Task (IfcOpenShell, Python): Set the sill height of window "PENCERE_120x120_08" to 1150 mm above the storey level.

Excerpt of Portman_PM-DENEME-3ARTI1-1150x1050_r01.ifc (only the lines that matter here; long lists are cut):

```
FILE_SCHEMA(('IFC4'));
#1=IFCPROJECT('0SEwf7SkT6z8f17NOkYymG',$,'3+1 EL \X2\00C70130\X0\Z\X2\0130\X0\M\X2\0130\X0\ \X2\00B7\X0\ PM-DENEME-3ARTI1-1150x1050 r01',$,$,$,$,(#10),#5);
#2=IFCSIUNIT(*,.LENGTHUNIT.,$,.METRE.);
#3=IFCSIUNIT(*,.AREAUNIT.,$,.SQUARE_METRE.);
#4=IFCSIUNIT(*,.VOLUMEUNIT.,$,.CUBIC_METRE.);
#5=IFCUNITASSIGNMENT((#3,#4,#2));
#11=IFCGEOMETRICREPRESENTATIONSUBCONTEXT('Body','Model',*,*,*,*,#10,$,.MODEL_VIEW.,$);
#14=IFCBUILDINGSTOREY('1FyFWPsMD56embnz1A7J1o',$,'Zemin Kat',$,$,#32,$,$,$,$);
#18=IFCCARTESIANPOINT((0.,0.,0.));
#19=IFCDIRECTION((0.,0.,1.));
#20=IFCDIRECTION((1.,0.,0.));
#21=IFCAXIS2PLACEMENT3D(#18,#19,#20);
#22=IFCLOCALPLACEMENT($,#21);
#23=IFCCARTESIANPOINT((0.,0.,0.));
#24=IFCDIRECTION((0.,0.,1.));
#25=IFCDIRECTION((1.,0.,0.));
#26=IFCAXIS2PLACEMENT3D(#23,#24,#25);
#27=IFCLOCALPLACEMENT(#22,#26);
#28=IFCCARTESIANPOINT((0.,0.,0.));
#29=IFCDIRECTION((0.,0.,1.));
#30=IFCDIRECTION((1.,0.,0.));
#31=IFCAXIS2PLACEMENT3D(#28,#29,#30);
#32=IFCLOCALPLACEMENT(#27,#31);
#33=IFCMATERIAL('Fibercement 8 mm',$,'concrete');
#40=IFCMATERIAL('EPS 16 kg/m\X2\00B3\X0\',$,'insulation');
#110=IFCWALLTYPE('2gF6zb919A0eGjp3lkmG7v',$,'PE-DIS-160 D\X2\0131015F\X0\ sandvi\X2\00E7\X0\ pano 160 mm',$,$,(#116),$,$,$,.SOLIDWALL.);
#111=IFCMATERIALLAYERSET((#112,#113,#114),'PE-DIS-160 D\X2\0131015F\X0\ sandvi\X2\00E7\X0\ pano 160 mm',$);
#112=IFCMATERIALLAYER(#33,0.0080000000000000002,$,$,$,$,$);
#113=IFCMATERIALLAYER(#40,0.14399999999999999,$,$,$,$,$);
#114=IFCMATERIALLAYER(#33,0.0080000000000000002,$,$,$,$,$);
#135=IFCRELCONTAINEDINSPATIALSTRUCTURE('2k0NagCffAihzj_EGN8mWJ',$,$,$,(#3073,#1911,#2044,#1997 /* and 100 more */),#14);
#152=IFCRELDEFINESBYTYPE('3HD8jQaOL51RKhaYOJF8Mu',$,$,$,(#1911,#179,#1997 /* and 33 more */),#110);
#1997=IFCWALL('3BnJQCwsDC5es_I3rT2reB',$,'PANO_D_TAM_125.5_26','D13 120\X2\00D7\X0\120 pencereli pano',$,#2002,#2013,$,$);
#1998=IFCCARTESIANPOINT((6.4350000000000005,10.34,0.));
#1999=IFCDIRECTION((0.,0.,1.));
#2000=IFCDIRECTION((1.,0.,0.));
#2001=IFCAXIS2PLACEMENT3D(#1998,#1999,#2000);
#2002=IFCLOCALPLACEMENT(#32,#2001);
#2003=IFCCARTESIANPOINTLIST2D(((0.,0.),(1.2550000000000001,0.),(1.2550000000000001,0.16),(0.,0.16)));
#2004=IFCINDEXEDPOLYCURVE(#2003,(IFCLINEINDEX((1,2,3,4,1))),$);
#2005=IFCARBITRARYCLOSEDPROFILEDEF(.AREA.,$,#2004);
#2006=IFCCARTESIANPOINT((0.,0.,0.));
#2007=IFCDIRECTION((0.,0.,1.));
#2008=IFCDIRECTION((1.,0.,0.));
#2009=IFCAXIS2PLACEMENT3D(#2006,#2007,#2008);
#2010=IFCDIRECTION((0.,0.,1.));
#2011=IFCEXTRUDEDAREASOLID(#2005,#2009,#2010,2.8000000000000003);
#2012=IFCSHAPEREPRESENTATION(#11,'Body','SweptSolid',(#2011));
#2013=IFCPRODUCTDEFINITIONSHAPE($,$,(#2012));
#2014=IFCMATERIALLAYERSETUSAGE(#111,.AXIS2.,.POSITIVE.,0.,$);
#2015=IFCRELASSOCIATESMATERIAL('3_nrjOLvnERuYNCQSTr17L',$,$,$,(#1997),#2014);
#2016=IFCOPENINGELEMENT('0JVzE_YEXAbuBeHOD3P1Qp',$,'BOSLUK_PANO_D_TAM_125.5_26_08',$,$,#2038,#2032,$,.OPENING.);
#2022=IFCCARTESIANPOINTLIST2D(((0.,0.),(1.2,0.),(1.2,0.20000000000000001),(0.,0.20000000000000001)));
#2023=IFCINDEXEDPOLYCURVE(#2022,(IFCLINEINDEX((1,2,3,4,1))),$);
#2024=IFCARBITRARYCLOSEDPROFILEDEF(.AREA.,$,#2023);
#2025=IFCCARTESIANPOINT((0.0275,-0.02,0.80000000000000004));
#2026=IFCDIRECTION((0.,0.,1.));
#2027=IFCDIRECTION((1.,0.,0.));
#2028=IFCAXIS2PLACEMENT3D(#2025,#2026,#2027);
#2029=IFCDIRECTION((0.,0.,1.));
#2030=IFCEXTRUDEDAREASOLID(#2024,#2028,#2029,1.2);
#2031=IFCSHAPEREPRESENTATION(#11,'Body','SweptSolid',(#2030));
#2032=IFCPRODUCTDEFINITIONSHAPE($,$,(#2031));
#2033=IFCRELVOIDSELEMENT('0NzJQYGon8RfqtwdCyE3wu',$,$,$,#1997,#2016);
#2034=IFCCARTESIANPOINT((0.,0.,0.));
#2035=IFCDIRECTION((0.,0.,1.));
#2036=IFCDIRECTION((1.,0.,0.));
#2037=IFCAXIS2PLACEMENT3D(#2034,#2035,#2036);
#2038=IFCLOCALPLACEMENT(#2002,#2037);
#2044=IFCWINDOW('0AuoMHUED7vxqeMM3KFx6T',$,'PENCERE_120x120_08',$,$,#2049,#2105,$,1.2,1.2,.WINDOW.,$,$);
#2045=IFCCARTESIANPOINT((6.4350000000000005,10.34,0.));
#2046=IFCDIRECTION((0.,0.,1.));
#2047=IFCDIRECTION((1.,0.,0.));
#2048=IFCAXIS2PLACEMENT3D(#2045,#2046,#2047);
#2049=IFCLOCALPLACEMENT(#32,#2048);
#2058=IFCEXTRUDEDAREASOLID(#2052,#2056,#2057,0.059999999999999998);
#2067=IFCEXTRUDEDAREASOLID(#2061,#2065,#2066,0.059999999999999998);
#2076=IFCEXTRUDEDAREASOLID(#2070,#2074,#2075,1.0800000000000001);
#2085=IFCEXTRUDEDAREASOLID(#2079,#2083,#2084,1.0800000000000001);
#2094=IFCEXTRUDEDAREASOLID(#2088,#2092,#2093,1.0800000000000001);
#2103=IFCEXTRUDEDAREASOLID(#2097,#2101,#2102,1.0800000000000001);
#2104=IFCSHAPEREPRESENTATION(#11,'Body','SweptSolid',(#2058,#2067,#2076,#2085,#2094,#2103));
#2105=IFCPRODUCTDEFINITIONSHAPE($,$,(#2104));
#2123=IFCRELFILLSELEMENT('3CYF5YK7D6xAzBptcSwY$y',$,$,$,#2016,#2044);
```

```python
import numpy as np
import ifcopenshell
import ifcopenshell.api.geometry
import ifcopenshell.geom
import ifcopenshell.util.element
import ifcopenshell.util.placement
import ifcopenshell.util.shape
import ifcopenshell.util.unit

model = ifcopenshell.open("Portman_PM-DENEME-3ARTI1-1150x1050_r01.ifc")
unit_scale = ifcopenshell.util.unit.calculate_unit_scale(model)

window = model.by_guid("0AuoMHUED7vxqeMM3KFx6T")
opening = window.FillsVoids[0].RelatingOpeningElement
storey = ifcopenshell.util.element.get_container(window, ifc_class="IfcBuildingStorey")
level = ifcopenshell.util.placement.get_local_placement(storey.ObjectPlacement)[2, 3]

# The opening's origin need not be at the sill, so measure its lowest point.
shape = ifcopenshell.geom.create_shape(ifcopenshell.geom.settings(), opening)
bottom = ifcopenshell.util.shape.get_shape_bottom_elevation(shape, shape.geometry) / unit_scale
dz = level + 1.15 - bottom

shift = np.array([0.0, 0.0, dz])
# The window is not placed relative to its opening, so move both.
for product in (opening, window):
    matrix = ifcopenshell.util.placement.get_local_placement(product.ObjectPlacement)
    matrix[:3, 3] += shift
    ifcopenshell.api.geometry.edit_object_placement(model, product=product, matrix=matrix, is_si=False)

print(f"moved by {dz * unit_scale:+.3f} m")

model.write("Portman_PM-DENEME-3ARTI1-1150x1050_r01_edited.ifc")
```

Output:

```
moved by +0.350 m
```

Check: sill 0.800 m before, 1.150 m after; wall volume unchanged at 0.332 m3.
